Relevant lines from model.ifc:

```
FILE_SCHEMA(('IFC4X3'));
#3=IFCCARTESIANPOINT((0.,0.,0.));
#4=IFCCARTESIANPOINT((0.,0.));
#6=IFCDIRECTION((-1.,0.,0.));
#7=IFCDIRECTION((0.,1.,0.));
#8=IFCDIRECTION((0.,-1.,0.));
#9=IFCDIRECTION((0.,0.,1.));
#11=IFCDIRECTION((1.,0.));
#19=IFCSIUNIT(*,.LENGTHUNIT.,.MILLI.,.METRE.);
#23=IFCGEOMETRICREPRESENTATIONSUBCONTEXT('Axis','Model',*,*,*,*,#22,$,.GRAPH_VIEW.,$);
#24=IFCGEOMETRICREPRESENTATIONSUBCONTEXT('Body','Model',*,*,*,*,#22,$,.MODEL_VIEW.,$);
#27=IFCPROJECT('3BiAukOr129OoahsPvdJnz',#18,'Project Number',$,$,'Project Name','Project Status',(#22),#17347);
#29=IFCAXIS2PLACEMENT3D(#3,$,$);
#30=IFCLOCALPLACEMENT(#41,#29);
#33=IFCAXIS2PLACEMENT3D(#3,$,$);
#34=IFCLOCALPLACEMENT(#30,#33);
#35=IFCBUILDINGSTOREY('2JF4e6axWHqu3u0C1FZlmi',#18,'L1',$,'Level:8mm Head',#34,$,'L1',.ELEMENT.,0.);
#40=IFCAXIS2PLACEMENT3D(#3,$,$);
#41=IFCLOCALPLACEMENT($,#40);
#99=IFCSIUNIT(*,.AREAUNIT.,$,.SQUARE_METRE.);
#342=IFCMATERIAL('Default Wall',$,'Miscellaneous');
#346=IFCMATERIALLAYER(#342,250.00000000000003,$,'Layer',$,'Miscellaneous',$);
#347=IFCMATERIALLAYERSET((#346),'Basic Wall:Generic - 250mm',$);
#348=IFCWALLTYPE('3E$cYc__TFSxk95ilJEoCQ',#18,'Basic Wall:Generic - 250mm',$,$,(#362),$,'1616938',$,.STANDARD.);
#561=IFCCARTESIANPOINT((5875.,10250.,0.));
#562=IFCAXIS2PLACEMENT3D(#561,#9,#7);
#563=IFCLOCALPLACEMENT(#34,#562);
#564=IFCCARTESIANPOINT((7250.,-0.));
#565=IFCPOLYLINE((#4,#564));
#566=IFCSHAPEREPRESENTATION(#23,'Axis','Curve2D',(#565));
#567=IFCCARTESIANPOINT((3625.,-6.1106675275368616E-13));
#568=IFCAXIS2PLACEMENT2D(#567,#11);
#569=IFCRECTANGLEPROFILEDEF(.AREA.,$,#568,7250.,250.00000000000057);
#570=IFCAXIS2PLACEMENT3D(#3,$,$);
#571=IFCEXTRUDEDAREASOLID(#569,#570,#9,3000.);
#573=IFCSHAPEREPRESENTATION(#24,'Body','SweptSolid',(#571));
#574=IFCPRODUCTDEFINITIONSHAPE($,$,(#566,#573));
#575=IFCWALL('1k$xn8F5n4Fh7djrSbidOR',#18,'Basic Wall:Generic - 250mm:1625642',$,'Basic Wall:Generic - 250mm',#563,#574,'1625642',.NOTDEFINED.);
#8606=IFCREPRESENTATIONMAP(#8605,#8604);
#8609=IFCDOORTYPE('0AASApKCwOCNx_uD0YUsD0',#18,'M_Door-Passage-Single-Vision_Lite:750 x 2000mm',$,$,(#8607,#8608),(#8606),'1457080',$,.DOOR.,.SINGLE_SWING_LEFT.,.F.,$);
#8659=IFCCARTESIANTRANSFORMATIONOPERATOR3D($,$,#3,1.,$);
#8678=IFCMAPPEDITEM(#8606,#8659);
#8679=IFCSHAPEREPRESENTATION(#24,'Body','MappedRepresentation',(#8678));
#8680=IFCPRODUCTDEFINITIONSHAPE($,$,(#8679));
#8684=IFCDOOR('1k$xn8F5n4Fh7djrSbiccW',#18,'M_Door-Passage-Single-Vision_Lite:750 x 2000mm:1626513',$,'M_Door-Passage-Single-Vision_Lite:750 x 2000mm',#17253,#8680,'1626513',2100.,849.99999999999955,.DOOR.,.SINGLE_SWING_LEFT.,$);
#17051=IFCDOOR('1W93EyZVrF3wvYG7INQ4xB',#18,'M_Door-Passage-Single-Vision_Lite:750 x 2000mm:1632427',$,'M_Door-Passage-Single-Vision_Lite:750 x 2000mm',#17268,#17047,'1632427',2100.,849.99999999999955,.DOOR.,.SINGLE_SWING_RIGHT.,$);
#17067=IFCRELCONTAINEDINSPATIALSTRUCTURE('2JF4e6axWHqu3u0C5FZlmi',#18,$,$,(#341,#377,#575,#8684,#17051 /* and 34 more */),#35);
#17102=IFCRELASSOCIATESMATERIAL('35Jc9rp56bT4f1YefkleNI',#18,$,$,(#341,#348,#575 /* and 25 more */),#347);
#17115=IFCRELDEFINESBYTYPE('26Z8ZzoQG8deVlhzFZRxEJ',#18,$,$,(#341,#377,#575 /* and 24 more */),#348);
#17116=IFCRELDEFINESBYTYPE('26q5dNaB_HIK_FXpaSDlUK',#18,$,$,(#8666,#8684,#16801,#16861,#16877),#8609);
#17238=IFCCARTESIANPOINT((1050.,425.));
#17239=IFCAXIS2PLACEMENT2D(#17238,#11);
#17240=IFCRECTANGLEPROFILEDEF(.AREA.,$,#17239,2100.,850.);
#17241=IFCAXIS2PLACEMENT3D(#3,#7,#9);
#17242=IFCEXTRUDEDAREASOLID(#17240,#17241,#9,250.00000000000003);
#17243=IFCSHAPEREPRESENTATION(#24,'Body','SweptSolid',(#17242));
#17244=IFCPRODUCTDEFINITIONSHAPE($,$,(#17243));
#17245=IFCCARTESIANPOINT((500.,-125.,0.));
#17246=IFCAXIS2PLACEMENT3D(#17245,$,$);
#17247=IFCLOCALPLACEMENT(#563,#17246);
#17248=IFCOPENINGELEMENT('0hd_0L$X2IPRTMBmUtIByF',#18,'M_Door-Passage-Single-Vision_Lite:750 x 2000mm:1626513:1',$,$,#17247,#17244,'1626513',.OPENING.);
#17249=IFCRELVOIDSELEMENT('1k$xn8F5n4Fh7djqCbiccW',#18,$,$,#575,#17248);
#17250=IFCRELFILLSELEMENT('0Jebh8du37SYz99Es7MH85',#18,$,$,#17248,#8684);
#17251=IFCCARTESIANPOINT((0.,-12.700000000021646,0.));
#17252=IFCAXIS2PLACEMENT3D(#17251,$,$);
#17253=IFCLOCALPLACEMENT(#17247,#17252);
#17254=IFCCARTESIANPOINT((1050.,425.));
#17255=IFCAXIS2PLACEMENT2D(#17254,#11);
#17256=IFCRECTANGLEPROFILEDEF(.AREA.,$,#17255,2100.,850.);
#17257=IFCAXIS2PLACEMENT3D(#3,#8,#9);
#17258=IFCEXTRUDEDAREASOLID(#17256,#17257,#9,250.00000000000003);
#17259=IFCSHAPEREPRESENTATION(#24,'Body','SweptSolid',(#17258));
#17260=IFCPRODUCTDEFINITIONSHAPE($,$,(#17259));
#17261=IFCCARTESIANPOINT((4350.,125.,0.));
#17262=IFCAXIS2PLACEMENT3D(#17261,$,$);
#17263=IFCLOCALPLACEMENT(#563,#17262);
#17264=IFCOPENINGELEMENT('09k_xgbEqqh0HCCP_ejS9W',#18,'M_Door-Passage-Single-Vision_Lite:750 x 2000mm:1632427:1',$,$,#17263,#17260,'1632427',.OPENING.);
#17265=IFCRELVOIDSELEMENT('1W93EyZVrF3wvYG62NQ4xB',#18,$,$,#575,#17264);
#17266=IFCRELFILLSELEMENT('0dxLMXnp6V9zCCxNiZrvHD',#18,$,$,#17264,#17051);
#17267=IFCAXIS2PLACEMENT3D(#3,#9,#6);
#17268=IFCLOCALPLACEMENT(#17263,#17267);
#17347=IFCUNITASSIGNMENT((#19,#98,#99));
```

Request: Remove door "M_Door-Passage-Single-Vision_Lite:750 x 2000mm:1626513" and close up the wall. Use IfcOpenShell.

```python
import ifcopenshell
import ifcopenshell.api.feature
import ifcopenshell.api.root
import ifcopenshell.geom
import ifcopenshell.util.shape

model = ifcopenshell.open("model.ifc")
settings = ifcopenshell.geom.settings()


def volume(element):
    """Net volume in cubic metres, openings subtracted."""
    shape = ifcopenshell.geom.create_shape(settings, element)
    return ifcopenshell.util.shape.get_volume(shape.geometry)


door = model.by_guid("1k$xn8F5n4Fh7djrSbiccW")
opening = door.FillsVoids[0].RelatingOpeningElement
wall = opening.VoidsElements[0].RelatingBuildingElement
before = volume(wall)

ifcopenshell.api.root.remove_product(model, product=door)
ifcopenshell.api.feature.remove_feature(model, feature=opening)

after = volume(wall)

print(f"wall volume {before:.3f} -> {after:.3f} m3")

model.write("model_edited.ifc")
```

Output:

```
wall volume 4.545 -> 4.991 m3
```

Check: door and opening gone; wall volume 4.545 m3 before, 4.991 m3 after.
